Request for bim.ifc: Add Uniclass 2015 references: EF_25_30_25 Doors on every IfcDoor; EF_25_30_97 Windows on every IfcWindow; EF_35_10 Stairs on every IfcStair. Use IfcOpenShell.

First a look at what the model holds.

```python
import ifcopenshell

model = ifcopenshell.open("bim.ifc")
print(model.schema)
print("classifications:", [c.Name for c in model.by_type("IfcClassification")])
for ifc_class in ("IfcDoor", "IfcRoof", "IfcStair", "IfcWall", "IfcWindow"):
    print(ifc_class, len(model.by_type(ifc_class)))
```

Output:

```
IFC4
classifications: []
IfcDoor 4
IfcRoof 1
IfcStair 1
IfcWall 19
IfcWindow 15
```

```python
import ifcopenshell
import ifcopenshell.api.classification

model = ifcopenshell.open("bim.ifc")

system = ifcopenshell.api.classification.add_classification(model, classification="Uniclass 2015")

codes = {
    "IfcDoor": ("EF_25_30_25", "Doors"),
    "IfcWindow": ("EF_25_30_97", "Windows"),
    "IfcStair": ("EF_35_10", "Stairs"),
}
for ifc_class, (code, name) in codes.items():
    products = model.by_type(ifc_class)
    ifcopenshell.api.classification.add_reference(
        model, products=products, classification=system, identification=code, name=name
    )
    print(code, len(products))

model.write("bim_edited.ifc")
```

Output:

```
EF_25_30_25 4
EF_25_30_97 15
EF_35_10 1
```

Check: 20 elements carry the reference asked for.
